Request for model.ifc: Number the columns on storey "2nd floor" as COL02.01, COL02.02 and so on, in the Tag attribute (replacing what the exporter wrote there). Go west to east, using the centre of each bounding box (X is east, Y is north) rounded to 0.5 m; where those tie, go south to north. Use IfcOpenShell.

First a look at what the model holds.

```python
import ifcopenshell
import ifcopenshell.util.element
import ifcopenshell.util.placement

model = ifcopenshell.open("model.ifc")
print(model.schema)
storey = next(s for s in model.by_type("IfcBuildingStorey") if s.Name == "2nd floor")
columns = [e for e in ifcopenshell.util.element.get_decomposition(storey) if e.is_a("IfcColumn")]
for e in sorted(columns, key=lambda e: e.id()):
    origin = ifcopenshell.util.placement.get_local_placement(e.ObjectPlacement)[:3, 3]
    print(e.id(), e.Tag, e.Name, origin.round(2) + 0.0, sep=" | ")
```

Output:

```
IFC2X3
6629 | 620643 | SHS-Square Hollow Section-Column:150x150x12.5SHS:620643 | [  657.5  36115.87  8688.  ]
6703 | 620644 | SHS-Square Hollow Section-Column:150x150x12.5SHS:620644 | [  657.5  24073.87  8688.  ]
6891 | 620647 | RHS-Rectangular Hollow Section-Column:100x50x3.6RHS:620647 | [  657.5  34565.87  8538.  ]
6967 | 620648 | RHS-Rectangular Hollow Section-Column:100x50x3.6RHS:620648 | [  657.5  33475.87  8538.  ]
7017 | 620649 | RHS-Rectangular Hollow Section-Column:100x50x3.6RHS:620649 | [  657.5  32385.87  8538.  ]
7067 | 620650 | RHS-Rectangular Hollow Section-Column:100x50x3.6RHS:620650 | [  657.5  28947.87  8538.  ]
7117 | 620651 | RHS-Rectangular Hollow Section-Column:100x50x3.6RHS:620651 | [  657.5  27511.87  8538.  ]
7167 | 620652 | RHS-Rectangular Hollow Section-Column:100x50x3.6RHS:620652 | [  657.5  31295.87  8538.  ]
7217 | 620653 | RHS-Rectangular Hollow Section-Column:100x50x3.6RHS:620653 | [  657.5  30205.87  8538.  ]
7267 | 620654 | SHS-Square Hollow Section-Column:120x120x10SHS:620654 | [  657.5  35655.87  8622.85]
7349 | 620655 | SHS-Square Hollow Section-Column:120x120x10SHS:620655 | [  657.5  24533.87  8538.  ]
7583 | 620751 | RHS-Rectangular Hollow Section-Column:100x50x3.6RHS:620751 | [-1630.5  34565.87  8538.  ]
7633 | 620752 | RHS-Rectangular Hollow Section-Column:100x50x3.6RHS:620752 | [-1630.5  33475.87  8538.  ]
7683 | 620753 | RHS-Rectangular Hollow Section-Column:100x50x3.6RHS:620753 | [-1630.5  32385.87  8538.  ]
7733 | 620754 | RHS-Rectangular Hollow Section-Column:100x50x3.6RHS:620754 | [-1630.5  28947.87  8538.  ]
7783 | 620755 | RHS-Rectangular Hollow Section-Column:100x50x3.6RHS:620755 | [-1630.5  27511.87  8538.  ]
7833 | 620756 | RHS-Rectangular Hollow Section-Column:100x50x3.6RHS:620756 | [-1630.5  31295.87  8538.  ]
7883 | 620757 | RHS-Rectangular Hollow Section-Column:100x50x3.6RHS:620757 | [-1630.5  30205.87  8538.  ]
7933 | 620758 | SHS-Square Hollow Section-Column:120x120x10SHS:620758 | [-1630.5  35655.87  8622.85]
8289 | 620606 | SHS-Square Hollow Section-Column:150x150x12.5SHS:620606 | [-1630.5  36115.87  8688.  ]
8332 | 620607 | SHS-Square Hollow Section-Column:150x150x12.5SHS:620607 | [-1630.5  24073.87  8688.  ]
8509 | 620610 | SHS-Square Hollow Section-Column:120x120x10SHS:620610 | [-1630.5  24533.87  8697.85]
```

```python
import ifcopenshell
import ifcopenshell.geom
import ifcopenshell.util.element
import ifcopenshell.util.shape

model = ifcopenshell.open("model.ifc")
settings = ifcopenshell.geom.settings()
settings.set("use-world-coords", True)


def centre(element):
    shape = ifcopenshell.geom.create_shape(settings, element)
    return ifcopenshell.util.shape.get_bbox_centroid(shape.geometry)


storey = next(s for s in model.by_type("IfcBuildingStorey") if s.Name == "2nd floor")
columns = [e for e in ifcopenshell.util.element.get_decomposition(storey) if e.is_a("IfcColumn")]

# Insertion points can sit at a corner or the storey origin, so sort by the geometry (in metres).
centres = {e: centre(e) for e in columns}
columns.sort(key=lambda e: (round(centres[e][0] / 0.5), centres[e][1]))

for i, e in enumerate(columns, start=1):
    number = f"COL02.{i:02d}"
    e.Tag = number
    print(e.id(), number)

model.write("model-out.ifc")
```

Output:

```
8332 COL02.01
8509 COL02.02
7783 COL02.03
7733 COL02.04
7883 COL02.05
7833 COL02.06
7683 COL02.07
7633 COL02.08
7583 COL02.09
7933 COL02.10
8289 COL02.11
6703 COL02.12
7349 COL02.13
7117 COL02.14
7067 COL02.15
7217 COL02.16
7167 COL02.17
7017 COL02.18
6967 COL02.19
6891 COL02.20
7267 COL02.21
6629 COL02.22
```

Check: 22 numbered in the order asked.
